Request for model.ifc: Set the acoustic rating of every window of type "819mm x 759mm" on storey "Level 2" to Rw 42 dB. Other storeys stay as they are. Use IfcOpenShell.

First a look at what the model holds.

```python
import ifcopenshell
import ifcopenshell.util.element

model = ifcopenshell.open("model.ifc")
print(model.schema)
storey = next(s for s in model.by_type("IfcBuildingStorey") if s.Name == "Level 2")
windows = [e for e in ifcopenshell.util.element.get_decomposition(storey) if e.is_a("IfcWindow")]
seen = {}
for e in windows:
    element_type = ifcopenshell.util.element.get_type(e)
    key = (element_type.Name if element_type != e and element_type else None, ifcopenshell.util.element.get_pset(e, "Pset_WindowCommon", "AcousticRating"))
    seen[key] = seen.get(key, 0) + 1
for (name, value), count in sorted(seen.items(), key=str):
    print(count, "x", name, "|", value)
```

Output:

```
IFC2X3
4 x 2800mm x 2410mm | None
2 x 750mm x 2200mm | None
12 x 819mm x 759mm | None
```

```python
import ifcopenshell
import ifcopenshell.api.pset
import ifcopenshell.util.element

model = ifcopenshell.open("model.ifc")

storey = next(s for s in model.by_type("IfcBuildingStorey") if s.Name == "Level 2")
windows = [e for e in ifcopenshell.util.element.get_decomposition(storey) if e.is_a("IfcWindow")]

count = 0
for e in windows:
    element_type = ifcopenshell.util.element.get_type(e)
    if element_type in (None, e) or element_type.Name != "819mm x 759mm":
        continue
    # add_pset returns the element's existing set when there is one.
    pset = ifcopenshell.api.pset.add_pset(model, product=e, name="Pset_WindowCommon")
    ifcopenshell.api.pset.edit_pset(model, pset=pset, properties={"AcousticRating": "Rw 42 dB"})
    count += 1

print(count, "windows updated")

model.write("model_v2.ifc")
```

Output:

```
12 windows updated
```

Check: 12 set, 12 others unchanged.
